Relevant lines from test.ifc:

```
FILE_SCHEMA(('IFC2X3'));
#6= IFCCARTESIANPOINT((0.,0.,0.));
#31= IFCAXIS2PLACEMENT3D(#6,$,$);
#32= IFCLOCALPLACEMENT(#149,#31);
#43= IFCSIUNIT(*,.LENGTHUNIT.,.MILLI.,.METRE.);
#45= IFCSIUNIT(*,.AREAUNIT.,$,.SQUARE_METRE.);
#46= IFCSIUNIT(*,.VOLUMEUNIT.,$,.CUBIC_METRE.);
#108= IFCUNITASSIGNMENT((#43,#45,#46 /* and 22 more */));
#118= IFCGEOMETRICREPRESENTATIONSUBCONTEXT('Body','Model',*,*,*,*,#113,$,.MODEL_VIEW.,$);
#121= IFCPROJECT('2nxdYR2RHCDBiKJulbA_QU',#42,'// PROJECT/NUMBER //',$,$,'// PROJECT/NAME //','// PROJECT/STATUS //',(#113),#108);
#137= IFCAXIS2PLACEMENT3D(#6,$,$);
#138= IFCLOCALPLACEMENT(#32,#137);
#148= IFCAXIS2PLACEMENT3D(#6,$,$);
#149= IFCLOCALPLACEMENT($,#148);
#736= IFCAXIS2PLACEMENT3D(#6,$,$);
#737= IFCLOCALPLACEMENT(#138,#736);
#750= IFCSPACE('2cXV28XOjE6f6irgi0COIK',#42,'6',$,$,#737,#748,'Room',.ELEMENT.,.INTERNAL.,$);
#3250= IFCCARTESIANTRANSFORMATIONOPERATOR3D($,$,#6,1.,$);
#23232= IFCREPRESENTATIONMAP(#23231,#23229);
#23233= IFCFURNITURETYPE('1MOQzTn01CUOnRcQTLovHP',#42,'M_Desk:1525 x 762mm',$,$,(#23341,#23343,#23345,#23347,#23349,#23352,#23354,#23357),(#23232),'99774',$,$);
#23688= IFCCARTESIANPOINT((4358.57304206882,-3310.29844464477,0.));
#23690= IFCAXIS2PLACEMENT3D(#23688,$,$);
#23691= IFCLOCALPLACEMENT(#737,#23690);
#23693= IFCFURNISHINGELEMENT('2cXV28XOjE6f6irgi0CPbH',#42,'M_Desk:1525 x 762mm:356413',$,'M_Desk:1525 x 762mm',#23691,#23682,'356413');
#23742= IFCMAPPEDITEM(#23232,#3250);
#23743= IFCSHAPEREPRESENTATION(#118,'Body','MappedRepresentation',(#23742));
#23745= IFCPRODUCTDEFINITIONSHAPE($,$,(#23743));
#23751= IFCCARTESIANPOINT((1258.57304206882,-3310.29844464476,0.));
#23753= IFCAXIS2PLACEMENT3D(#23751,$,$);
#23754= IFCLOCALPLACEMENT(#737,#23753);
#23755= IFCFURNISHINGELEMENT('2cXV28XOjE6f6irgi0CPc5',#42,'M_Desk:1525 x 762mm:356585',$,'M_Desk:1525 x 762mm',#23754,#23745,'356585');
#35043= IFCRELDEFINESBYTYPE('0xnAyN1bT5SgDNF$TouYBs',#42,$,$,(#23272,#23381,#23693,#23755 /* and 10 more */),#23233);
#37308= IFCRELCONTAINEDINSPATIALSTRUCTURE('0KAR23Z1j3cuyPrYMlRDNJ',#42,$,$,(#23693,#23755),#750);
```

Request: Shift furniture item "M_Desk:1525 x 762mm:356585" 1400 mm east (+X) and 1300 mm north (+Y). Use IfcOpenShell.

```python
import ifcopenshell
import ifcopenshell.api.geometry
import ifcopenshell.util.placement

model = ifcopenshell.open("test.ifc")

item = model.by_id(23755)
matrix = ifcopenshell.util.placement.get_local_placement(item.ObjectPlacement)
matrix[0, 3] += 1400.0
matrix[1, 3] += 1300.0
ifcopenshell.api.geometry.edit_object_placement(model, product=item, matrix=matrix, is_si=False)

print(ifcopenshell.util.placement.get_local_placement(item.ObjectPlacement).round(3) + 0.0)

model.write("test_rev.ifc")
```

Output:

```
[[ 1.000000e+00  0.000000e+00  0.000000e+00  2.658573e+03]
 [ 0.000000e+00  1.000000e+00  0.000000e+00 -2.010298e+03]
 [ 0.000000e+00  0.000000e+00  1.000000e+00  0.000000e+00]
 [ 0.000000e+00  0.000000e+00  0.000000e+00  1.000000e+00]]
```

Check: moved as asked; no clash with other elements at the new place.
